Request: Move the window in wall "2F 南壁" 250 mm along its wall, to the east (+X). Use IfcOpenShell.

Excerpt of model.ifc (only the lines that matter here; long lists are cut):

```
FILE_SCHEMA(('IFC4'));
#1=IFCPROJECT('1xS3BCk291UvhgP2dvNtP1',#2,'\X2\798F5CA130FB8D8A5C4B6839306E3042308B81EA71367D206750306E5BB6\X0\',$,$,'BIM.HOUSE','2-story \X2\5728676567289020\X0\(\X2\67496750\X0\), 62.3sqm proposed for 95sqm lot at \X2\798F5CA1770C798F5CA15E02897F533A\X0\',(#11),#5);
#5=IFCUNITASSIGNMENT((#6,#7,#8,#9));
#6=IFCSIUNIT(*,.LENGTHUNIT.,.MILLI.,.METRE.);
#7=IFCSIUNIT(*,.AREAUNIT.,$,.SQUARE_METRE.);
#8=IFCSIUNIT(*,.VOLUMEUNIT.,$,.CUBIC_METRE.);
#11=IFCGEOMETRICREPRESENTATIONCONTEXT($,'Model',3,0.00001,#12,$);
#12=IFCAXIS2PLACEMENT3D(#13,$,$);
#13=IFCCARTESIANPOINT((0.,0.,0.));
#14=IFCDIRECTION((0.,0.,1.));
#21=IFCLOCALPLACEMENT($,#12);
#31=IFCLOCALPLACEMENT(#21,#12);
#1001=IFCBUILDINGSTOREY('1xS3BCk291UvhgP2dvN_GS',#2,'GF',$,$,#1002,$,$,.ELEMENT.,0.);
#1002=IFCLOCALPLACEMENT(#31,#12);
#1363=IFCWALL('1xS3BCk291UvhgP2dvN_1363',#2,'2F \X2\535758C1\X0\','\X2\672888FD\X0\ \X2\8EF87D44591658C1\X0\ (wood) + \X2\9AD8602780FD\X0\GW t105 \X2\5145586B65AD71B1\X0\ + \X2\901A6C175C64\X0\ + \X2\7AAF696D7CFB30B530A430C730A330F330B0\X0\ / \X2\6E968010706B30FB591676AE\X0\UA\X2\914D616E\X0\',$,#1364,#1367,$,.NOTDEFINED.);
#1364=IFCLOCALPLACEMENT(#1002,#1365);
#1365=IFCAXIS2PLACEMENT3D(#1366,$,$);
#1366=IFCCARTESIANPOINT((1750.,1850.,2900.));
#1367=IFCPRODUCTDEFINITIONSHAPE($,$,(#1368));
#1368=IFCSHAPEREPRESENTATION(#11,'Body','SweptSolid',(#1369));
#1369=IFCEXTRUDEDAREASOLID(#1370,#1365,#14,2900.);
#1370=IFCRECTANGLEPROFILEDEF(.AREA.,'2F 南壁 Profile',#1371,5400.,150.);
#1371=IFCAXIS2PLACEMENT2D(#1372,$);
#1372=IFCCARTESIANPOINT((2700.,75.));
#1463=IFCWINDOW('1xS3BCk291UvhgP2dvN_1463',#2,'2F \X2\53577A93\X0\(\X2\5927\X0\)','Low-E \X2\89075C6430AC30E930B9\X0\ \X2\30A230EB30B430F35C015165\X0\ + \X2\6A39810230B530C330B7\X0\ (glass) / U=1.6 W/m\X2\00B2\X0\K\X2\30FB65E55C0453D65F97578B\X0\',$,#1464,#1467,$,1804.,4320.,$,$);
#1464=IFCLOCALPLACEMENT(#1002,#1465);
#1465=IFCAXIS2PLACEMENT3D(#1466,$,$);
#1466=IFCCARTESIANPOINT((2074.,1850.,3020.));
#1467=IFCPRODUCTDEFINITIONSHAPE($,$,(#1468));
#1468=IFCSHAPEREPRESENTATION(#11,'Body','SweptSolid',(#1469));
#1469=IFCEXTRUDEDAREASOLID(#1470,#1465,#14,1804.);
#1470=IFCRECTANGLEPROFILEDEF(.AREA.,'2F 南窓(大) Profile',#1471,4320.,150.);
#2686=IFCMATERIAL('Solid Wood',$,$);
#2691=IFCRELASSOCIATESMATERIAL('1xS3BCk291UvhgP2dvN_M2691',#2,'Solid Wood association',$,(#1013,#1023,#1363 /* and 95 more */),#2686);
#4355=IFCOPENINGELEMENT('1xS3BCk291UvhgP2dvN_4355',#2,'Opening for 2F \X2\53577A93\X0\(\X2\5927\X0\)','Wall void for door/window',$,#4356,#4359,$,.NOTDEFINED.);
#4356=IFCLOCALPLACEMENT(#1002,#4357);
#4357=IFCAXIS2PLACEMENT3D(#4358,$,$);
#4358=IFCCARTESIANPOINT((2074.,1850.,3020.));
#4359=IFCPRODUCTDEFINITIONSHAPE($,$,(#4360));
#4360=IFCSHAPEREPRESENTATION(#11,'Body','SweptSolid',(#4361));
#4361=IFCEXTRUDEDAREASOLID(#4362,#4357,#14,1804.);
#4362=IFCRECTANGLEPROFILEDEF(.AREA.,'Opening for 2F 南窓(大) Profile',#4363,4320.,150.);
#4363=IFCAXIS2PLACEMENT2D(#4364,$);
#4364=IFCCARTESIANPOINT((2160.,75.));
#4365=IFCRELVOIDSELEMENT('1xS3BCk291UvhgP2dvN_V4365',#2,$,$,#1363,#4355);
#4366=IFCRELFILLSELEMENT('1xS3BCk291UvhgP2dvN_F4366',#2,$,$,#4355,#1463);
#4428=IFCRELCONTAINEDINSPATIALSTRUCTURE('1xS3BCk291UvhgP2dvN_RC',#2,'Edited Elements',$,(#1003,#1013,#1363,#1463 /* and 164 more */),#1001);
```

```python
import ifcopenshell
import ifcopenshell.api.geometry
import ifcopenshell.util.placement

model = ifcopenshell.open("model.ifc")

window = model.by_guid("1xS3BCk291UvhgP2dvN_1463")
opening = window.FillsVoids[0].RelatingOpeningElement
wall = opening.VoidsElements[0].RelatingBuildingElement

wall_matrix = ifcopenshell.util.placement.get_local_placement(wall.ObjectPlacement)
shift = wall_matrix[:3, 0] * 250.0
before = ifcopenshell.util.placement.get_local_placement(window.ObjectPlacement)[:3, 3].copy()

# The window is not placed relative to its opening, so move both.
for product in (opening, window):
    matrix = ifcopenshell.util.placement.get_local_placement(product.ObjectPlacement)
    matrix[:3, 3] += shift
    ifcopenshell.api.geometry.edit_object_placement(model, product=product, matrix=matrix, is_si=False)

after = ifcopenshell.util.placement.get_local_placement(window.ObjectPlacement)[:3, 3]
print("window moved by", (after - before).round(3) + 0.0)

model.write("model-out.ifc")
```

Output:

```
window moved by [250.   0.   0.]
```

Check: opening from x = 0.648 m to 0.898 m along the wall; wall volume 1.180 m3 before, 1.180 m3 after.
